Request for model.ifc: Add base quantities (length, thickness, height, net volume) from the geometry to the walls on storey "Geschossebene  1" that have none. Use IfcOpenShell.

First a look at what the model holds.

```python
import ifcopenshell
import ifcopenshell.util.element
import ifcopenshell.util.unit

model = ifcopenshell.open("model.ifc")
print(model.schema)
for unit_type in ("LENGTHUNIT", "AREAUNIT", "VOLUMEUNIT"):
    print(unit_type, ifcopenshell.util.unit.calculate_unit_scale(model, unit_type))
storey = next(s for s in model.by_type("IfcBuildingStorey") if s.Name == "Geschossebene  1")
walls = [e for e in ifcopenshell.util.element.get_decomposition(storey) if e.is_a("IfcWall")]
for e in sorted(walls, key=lambda e: e.id()):
    print(e.id(), e.is_a(), e.Name, list(ifcopenshell.util.element.get_psets(e, qtos_only=True)), sep=" | ")
```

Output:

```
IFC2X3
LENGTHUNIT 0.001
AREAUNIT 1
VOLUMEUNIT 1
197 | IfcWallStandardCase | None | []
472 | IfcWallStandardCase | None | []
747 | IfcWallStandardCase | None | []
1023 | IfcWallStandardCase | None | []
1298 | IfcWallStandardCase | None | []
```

```python
import ifcopenshell
import ifcopenshell.api.pset
import ifcopenshell.geom
import ifcopenshell.util.element
import ifcopenshell.util.shape
import ifcopenshell.util.unit

model = ifcopenshell.open("model.ifc")
unit_scale = ifcopenshell.util.unit.calculate_unit_scale(model)
volume_scale = ifcopenshell.util.unit.calculate_unit_scale(model, "VOLUMEUNIT")
settings = ifcopenshell.geom.settings()

storey = next(s for s in model.by_type("IfcBuildingStorey") if s.Name == "Geschossebene  1")
walls = [e for e in ifcopenshell.util.element.get_decomposition(storey) if e.is_a("IfcWall")]

for e in sorted(walls, key=lambda e: e.id()):
    if ifcopenshell.util.element.get_psets(e, qtos_only=True, should_inherit=False):
        continue
    # Geometry comes back in metres, in the element's own axes.
    shape = ifcopenshell.geom.create_shape(settings, e)
    values = {
        "Length": ifcopenshell.util.shape.get_x(shape.geometry) / unit_scale,
        "Width": ifcopenshell.util.shape.get_y(shape.geometry) / unit_scale,
        "Height": ifcopenshell.util.shape.get_z(shape.geometry) / unit_scale,
        "NetVolume": ifcopenshell.util.shape.get_volume(shape.geometry) / volume_scale,
    }
    qto = ifcopenshell.api.pset.add_qto(model, product=e, name="BaseQuantities")
    ifcopenshell.api.pset.edit_qto(model, qto=qto, properties=values)
    print(e.id(), {k: round(v, 3) for k, v in values.items()})

model.write("model_updated.ifc")
```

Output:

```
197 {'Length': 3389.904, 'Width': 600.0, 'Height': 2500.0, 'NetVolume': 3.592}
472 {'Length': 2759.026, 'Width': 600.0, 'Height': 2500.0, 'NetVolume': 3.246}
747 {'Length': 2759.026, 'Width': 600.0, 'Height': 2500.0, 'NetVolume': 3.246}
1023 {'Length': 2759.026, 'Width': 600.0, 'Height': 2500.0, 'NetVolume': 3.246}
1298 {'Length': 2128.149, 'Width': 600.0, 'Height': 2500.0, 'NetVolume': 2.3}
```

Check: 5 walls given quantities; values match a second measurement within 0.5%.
